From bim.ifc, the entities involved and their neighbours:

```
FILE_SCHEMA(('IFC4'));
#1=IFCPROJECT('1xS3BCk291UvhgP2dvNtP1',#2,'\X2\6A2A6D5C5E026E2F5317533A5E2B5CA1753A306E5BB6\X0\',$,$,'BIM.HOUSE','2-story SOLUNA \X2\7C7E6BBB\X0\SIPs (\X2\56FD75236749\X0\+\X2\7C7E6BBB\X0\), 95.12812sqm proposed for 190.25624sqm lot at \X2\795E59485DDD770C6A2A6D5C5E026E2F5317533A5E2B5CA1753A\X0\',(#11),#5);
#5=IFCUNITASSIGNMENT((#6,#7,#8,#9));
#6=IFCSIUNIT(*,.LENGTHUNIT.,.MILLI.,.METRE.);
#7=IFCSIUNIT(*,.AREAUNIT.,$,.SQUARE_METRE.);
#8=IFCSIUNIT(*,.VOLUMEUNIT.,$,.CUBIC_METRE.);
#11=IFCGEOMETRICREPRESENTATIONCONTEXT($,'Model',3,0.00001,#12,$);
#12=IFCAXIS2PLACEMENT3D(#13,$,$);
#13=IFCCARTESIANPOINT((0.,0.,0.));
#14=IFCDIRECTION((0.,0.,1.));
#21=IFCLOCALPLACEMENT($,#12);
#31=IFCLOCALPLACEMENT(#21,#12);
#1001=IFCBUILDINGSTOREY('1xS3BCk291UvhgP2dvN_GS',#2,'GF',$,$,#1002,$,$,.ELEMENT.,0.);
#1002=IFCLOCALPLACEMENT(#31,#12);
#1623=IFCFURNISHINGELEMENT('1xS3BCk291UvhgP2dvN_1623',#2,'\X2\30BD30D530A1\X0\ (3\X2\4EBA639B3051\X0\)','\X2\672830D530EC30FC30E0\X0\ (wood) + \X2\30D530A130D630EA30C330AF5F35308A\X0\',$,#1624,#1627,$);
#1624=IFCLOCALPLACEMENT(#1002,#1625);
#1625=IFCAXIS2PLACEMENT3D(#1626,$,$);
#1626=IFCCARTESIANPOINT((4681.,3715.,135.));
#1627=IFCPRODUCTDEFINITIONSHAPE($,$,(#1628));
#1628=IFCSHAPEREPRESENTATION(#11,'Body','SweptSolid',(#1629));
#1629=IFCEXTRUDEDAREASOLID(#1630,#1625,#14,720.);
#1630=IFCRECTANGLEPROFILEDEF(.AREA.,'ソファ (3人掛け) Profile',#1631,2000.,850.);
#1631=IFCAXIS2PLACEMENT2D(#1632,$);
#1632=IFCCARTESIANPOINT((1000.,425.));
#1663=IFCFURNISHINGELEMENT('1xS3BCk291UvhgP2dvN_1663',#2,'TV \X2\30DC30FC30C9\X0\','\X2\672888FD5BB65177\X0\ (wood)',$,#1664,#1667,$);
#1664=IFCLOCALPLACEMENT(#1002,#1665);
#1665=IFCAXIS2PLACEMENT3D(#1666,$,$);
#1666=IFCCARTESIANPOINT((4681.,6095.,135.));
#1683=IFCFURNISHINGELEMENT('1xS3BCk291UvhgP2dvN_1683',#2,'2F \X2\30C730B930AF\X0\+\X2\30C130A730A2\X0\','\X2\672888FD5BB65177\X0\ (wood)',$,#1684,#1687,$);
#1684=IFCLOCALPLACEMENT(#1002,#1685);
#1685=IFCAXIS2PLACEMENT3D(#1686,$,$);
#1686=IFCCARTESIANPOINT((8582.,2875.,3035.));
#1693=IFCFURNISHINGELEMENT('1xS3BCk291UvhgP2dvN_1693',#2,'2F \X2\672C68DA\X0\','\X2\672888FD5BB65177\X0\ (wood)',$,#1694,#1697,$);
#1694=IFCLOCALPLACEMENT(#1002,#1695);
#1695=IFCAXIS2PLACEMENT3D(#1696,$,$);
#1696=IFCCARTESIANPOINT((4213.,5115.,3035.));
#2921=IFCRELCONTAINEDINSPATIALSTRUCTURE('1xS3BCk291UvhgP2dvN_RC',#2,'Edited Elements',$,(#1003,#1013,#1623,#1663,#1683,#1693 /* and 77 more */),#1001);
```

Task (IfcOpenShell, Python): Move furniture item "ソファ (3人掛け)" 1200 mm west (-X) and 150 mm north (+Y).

```python
import ifcopenshell
import ifcopenshell.api.geometry
import ifcopenshell.util.placement
import ifcopenshell.util.unit

model = ifcopenshell.open("bim.ifc")
unit_scale = ifcopenshell.util.unit.calculate_unit_scale(model)

item = model.by_id(1623)
matrix = ifcopenshell.util.placement.get_local_placement(item.ObjectPlacement)
matrix[0, 3] -= 1.2 / unit_scale
matrix[1, 3] += 0.15 / unit_scale
ifcopenshell.api.geometry.edit_object_placement(model, product=item, matrix=matrix, is_si=False)

print(ifcopenshell.util.placement.get_local_placement(item.ObjectPlacement).round(3) + 0.0)

model.write("bim_updated.ifc")
```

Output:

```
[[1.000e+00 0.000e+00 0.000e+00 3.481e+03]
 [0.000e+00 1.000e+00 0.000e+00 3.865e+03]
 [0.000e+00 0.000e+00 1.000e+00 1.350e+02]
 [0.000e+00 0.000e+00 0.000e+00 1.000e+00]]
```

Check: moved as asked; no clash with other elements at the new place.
